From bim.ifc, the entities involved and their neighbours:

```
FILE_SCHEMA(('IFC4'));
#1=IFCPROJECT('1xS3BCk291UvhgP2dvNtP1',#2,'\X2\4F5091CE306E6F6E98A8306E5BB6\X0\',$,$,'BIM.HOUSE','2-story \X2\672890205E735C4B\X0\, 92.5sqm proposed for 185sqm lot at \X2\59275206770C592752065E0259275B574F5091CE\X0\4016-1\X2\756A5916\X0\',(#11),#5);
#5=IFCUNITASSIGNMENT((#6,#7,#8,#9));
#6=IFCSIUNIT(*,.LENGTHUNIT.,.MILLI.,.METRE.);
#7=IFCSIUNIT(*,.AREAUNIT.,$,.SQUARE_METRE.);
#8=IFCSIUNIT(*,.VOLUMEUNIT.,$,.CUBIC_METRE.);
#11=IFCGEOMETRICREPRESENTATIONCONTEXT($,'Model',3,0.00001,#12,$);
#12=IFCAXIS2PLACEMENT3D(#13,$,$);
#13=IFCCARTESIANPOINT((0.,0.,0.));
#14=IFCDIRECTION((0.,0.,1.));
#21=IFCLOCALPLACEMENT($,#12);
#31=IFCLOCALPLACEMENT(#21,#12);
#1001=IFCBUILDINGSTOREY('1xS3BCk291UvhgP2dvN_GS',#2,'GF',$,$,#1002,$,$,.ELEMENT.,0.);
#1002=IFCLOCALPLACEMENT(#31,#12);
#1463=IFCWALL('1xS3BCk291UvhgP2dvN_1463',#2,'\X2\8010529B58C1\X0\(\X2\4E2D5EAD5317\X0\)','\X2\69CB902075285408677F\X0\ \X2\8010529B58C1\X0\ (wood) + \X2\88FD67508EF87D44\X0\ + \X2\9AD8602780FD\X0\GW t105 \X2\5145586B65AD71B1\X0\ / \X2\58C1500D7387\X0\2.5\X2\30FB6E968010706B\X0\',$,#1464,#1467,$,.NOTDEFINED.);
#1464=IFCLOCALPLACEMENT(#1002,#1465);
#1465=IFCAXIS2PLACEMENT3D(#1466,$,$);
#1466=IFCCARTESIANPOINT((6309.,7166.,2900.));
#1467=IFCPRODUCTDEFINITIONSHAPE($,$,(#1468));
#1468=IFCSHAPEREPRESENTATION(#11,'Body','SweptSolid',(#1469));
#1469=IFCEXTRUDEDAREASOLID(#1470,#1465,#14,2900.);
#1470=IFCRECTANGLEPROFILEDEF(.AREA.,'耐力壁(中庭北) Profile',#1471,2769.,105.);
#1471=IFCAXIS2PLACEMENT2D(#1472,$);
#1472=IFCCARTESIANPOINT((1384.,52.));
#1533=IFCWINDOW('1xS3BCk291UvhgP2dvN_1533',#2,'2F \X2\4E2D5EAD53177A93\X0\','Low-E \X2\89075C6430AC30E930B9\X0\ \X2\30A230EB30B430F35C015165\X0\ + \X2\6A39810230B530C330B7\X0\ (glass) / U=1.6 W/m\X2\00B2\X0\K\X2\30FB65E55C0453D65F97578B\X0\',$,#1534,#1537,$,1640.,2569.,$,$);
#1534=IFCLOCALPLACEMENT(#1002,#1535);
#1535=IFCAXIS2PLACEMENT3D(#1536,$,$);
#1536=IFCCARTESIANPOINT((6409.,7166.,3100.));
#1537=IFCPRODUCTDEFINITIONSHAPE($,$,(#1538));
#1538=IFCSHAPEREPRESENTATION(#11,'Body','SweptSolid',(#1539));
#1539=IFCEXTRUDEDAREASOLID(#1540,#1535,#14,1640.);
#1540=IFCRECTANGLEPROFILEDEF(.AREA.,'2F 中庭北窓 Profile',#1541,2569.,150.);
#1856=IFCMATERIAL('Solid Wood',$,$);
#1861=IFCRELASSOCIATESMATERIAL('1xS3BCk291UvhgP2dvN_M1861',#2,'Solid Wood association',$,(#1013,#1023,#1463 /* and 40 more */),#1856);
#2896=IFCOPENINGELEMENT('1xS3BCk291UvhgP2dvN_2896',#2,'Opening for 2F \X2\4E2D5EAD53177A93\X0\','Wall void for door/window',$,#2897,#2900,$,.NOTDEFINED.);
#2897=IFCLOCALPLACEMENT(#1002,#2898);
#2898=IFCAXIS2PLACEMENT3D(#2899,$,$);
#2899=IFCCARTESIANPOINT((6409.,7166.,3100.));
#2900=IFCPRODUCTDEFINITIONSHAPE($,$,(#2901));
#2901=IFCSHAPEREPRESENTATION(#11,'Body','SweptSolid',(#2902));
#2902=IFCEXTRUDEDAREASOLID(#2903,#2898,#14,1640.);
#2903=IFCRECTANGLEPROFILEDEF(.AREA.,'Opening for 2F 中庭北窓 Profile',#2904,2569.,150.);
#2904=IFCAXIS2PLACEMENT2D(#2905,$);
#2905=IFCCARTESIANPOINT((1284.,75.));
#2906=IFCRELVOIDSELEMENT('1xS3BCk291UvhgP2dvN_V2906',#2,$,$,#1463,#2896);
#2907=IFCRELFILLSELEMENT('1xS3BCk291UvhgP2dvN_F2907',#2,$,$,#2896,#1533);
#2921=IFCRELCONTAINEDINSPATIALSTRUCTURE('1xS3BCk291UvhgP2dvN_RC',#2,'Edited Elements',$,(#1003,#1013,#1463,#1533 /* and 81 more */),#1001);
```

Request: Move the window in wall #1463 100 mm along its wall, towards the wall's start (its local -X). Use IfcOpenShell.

```python
import ifcopenshell
import ifcopenshell.api.geometry
import ifcopenshell.util.placement

model = ifcopenshell.open("bim.ifc")

window = model.by_guid("1xS3BCk291UvhgP2dvN_1533")
opening = window.FillsVoids[0].RelatingOpeningElement
wall = opening.VoidsElements[0].RelatingBuildingElement

wall_matrix = ifcopenshell.util.placement.get_local_placement(wall.ObjectPlacement)
shift = wall_matrix[:3, 0] * -100.0
before = ifcopenshell.util.placement.get_local_placement(window.ObjectPlacement)[:3, 3].copy()

# The window is not placed relative to its opening, so move both.
for product in (opening, window):
    matrix = ifcopenshell.util.placement.get_local_placement(product.ObjectPlacement)
    matrix[:3, 3] += shift
    ifcopenshell.api.geometry.edit_object_placement(model, product=product, matrix=matrix, is_si=False)

after = ifcopenshell.util.placement.get_local_placement(window.ObjectPlacement)[:3, 3]
print("window moved by", (after - before).round(3) + 0.0)

model.write("bim_edited.ifc")
```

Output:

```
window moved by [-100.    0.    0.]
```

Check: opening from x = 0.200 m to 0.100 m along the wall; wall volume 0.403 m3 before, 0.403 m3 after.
